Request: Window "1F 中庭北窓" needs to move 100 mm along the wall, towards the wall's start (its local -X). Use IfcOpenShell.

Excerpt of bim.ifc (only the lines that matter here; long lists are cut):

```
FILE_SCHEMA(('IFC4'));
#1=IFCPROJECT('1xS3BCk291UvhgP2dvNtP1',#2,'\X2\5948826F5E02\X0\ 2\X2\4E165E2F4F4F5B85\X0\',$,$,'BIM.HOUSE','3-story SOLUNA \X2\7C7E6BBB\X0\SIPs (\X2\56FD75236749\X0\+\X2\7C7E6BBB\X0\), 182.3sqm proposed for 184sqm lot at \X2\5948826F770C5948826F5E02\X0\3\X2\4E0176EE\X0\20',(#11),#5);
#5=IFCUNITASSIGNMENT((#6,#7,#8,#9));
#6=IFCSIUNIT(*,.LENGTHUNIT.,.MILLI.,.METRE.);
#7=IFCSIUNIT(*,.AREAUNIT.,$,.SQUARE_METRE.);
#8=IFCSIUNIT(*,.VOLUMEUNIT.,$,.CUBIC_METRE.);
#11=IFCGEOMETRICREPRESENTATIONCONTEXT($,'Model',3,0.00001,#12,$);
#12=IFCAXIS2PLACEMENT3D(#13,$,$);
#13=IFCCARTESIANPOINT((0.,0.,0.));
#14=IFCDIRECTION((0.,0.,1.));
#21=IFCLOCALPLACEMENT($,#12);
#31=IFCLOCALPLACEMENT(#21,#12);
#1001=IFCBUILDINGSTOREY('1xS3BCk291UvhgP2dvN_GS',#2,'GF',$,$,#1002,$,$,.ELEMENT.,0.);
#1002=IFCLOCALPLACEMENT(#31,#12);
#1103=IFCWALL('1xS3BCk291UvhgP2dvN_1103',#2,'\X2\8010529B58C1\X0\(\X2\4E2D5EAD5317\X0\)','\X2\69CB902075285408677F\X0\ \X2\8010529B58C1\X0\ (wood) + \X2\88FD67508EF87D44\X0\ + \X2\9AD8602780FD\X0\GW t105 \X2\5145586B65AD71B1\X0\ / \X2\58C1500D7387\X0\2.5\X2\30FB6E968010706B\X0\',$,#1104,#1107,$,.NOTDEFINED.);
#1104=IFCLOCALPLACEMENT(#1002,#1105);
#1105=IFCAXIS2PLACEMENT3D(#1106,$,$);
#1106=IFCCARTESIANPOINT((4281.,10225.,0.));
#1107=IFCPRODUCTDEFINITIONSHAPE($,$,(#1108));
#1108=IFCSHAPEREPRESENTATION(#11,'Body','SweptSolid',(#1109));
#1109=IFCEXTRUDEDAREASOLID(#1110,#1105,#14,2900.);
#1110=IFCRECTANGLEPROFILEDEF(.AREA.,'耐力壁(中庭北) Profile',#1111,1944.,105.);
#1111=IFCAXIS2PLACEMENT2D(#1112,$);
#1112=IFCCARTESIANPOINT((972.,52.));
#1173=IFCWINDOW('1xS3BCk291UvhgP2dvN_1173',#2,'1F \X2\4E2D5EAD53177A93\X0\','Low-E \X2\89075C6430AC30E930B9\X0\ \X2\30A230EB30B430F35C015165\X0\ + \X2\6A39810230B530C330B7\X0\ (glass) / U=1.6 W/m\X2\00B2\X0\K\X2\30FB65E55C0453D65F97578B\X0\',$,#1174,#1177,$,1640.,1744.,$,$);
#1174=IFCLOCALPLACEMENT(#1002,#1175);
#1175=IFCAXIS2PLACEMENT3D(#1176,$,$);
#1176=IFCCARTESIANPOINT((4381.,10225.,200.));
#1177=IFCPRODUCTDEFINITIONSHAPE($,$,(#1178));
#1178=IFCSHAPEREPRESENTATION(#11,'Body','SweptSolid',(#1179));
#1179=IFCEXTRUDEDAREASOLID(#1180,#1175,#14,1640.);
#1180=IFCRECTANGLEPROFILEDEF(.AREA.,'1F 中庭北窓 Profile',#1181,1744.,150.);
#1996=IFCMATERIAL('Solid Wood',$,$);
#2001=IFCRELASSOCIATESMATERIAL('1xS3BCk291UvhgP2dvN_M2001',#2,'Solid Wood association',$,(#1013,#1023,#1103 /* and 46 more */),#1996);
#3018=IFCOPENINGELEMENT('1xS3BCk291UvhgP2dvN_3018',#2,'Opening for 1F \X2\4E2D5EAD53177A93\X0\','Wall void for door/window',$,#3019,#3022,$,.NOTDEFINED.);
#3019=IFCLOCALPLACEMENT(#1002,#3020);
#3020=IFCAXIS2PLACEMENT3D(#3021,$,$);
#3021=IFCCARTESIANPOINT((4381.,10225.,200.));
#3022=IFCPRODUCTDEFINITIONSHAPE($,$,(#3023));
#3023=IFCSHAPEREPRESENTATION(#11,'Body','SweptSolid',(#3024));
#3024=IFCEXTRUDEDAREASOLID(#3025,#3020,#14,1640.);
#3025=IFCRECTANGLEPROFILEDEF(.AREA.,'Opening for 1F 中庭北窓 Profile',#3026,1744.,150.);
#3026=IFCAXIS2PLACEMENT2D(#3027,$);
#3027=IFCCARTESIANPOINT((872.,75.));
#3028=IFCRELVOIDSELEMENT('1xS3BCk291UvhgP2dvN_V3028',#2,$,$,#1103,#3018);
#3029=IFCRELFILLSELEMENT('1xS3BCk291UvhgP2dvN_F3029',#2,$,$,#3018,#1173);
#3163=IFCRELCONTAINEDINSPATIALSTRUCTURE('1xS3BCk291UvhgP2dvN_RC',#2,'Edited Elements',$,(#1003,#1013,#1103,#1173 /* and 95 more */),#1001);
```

```python
import ifcopenshell
import ifcopenshell.api.geometry
import ifcopenshell.util.placement

model = ifcopenshell.open("bim.ifc")

window = model.by_guid("1xS3BCk291UvhgP2dvN_1173")
opening = window.FillsVoids[0].RelatingOpeningElement
wall = opening.VoidsElements[0].RelatingBuildingElement

wall_matrix = ifcopenshell.util.placement.get_local_placement(wall.ObjectPlacement)
shift = wall_matrix[:3, 0] * -100.0
before = ifcopenshell.util.placement.get_local_placement(window.ObjectPlacement)[:3, 3].copy()

# The window is not placed relative to its opening, so move both.
for product in (opening, window):
    matrix = ifcopenshell.util.placement.get_local_placement(product.ObjectPlacement)
    matrix[:3, 3] += shift
    ifcopenshell.api.geometry.edit_object_placement(model, product=product, matrix=matrix, is_si=False)

after = ifcopenshell.util.placement.get_local_placement(window.ObjectPlacement)[:3, 3]
print("window moved by", (after - before).round(3) + 0.0)

model.write("bim_rev.ifc")
```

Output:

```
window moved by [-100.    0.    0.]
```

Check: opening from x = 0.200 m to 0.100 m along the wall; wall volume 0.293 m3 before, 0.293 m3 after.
